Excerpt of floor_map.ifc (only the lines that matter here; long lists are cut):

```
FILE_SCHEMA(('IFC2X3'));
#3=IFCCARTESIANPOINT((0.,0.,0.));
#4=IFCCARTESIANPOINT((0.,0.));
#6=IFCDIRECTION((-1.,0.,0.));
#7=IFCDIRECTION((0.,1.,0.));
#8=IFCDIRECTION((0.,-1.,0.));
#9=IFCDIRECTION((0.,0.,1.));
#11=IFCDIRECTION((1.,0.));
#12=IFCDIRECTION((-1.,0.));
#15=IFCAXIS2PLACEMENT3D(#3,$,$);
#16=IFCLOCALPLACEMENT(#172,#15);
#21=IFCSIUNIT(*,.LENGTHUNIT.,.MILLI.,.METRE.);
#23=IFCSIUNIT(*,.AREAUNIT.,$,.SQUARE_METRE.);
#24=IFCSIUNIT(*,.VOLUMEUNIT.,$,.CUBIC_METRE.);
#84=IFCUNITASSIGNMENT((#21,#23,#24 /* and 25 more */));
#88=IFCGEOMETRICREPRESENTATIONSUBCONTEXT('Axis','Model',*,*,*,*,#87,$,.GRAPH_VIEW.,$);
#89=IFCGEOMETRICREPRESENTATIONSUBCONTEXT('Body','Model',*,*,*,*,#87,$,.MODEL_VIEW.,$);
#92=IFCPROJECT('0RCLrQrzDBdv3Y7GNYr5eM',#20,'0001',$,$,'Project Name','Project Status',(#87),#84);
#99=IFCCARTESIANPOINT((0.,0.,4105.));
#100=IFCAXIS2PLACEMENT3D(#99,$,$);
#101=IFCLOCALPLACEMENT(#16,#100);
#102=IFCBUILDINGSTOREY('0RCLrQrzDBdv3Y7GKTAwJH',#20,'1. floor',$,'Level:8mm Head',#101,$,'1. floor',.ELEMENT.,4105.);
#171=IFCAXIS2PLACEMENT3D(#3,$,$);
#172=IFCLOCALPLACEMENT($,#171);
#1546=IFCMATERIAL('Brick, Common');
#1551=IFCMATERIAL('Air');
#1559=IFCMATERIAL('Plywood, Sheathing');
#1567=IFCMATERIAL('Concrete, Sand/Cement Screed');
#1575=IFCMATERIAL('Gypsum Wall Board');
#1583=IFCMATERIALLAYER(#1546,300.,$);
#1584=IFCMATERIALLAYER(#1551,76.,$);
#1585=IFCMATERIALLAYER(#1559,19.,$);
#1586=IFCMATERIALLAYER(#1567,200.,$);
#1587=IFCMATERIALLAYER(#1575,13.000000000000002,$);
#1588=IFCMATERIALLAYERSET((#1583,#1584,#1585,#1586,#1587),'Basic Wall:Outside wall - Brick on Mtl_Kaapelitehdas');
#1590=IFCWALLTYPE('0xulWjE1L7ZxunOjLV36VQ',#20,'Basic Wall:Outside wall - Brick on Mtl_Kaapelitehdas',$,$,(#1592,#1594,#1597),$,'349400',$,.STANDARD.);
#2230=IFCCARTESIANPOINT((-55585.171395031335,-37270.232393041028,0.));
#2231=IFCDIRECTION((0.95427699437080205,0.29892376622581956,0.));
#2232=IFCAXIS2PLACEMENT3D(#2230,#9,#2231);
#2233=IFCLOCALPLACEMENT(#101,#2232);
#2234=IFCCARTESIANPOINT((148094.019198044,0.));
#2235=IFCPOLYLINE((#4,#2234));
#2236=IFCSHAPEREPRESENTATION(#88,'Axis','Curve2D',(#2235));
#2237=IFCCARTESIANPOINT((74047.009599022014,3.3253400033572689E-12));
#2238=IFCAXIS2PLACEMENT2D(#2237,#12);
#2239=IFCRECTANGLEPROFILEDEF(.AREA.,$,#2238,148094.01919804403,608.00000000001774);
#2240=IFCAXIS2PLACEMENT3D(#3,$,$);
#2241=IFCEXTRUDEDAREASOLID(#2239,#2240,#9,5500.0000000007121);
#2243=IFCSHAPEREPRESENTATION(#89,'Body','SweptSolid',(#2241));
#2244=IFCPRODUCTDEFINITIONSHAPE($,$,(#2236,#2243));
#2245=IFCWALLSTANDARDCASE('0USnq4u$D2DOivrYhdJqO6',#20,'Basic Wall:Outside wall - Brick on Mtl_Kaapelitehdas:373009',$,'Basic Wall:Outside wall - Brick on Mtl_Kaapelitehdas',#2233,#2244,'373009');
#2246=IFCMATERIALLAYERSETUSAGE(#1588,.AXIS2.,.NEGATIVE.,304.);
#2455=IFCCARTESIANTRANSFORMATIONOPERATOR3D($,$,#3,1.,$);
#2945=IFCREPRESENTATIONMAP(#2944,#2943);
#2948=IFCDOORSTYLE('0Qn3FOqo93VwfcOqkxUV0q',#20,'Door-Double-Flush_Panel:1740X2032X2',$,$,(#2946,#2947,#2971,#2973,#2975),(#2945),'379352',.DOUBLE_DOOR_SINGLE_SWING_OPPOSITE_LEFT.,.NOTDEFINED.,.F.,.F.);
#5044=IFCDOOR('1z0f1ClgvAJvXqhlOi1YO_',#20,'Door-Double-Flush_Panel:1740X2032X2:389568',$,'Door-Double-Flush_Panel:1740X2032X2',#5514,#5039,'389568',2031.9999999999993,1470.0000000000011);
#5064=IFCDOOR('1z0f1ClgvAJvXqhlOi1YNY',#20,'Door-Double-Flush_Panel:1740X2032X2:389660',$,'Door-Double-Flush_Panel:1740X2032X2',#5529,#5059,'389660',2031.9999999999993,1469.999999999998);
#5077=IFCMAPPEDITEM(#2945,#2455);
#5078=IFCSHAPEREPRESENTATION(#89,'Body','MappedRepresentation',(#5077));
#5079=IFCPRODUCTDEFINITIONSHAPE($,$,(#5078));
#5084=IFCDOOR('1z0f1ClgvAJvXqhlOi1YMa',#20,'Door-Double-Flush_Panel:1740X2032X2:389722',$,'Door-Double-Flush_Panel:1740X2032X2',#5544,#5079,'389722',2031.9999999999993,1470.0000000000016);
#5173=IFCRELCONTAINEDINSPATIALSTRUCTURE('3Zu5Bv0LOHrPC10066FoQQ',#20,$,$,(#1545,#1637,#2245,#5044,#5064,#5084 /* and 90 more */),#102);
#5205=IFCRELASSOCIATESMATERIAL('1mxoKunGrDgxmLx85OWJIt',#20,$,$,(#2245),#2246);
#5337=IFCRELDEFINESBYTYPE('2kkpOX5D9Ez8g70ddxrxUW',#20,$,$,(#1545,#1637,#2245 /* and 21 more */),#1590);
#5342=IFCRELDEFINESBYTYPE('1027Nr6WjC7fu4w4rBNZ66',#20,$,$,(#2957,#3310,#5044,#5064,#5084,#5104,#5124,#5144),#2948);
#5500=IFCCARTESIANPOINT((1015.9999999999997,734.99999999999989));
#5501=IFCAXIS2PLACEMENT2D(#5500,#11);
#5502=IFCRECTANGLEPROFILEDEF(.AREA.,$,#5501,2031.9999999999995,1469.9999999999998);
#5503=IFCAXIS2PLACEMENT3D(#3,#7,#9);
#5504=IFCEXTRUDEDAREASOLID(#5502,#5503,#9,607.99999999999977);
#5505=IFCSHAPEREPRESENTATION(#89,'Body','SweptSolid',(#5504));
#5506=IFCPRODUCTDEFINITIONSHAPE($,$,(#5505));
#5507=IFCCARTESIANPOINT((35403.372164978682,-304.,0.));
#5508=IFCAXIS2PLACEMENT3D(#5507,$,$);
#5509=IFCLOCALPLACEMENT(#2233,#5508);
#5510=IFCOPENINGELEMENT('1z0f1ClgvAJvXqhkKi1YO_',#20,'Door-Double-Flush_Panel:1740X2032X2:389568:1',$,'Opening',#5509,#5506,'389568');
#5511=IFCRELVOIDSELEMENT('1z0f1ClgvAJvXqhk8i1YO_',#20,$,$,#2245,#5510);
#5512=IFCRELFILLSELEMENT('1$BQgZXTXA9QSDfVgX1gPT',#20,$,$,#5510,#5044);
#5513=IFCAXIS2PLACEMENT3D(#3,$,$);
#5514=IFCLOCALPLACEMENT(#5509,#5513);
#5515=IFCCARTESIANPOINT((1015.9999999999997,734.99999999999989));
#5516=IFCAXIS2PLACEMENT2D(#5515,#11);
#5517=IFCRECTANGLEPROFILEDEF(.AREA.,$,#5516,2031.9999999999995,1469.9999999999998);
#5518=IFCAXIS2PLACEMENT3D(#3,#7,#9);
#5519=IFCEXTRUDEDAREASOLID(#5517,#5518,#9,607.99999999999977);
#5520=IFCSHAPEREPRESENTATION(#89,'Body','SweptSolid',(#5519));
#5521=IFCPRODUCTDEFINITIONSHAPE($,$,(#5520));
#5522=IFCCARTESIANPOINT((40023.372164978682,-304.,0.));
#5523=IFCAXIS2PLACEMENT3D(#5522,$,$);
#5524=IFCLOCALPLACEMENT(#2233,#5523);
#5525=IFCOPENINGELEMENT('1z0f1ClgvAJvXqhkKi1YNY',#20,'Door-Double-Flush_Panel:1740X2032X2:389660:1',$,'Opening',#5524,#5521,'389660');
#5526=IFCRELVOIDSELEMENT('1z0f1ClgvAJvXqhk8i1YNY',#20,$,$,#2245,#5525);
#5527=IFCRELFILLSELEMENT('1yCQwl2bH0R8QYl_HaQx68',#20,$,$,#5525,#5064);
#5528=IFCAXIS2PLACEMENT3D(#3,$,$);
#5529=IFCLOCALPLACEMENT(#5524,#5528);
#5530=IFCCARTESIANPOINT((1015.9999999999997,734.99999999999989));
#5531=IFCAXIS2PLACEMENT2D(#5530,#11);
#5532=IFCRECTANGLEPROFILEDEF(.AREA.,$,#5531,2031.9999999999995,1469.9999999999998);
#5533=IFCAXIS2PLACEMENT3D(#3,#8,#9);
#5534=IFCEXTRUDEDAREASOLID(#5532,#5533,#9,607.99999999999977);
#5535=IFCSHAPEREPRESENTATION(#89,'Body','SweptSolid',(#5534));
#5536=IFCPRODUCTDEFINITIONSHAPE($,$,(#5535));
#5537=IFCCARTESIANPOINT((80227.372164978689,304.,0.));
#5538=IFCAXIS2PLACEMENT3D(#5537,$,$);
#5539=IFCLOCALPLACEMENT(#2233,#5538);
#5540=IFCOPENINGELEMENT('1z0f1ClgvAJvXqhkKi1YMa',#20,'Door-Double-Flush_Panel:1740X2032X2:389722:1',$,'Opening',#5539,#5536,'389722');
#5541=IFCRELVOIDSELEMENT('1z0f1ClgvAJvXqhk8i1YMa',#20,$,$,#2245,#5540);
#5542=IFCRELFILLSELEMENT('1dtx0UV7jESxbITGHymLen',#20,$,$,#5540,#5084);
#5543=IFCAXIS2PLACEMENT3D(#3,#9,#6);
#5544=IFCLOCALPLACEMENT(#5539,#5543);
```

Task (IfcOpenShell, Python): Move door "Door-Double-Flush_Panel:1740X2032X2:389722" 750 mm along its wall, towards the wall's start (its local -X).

```python
import ifcopenshell
import ifcopenshell.api.geometry
import ifcopenshell.util.placement

model = ifcopenshell.open("floor_map.ifc")

door = model.by_guid("1z0f1ClgvAJvXqhlOi1YMa")
opening = door.FillsVoids[0].RelatingOpeningElement
wall = opening.VoidsElements[0].RelatingBuildingElement

wall_matrix = ifcopenshell.util.placement.get_local_placement(wall.ObjectPlacement)
shift = wall_matrix[:3, 0] * -750.0
before = ifcopenshell.util.placement.get_local_placement(door.ObjectPlacement)[:3, 3].copy()

# The door is placed relative to its opening, so it follows when the opening moves.
matrix = ifcopenshell.util.placement.get_local_placement(opening.ObjectPlacement)
matrix[:3, 3] += shift
ifcopenshell.api.geometry.edit_object_placement(
    model, product=opening, matrix=matrix, is_si=False, should_transform_children=True
)

after = ifcopenshell.util.placement.get_local_placement(door.ObjectPlacement)[:3, 3]
print("door moved by", (after - before).round(3) + 0.0)

model.write("floor_map_v2.ifc")
```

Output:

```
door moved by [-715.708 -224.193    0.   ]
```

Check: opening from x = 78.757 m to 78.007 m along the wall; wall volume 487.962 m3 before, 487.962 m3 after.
